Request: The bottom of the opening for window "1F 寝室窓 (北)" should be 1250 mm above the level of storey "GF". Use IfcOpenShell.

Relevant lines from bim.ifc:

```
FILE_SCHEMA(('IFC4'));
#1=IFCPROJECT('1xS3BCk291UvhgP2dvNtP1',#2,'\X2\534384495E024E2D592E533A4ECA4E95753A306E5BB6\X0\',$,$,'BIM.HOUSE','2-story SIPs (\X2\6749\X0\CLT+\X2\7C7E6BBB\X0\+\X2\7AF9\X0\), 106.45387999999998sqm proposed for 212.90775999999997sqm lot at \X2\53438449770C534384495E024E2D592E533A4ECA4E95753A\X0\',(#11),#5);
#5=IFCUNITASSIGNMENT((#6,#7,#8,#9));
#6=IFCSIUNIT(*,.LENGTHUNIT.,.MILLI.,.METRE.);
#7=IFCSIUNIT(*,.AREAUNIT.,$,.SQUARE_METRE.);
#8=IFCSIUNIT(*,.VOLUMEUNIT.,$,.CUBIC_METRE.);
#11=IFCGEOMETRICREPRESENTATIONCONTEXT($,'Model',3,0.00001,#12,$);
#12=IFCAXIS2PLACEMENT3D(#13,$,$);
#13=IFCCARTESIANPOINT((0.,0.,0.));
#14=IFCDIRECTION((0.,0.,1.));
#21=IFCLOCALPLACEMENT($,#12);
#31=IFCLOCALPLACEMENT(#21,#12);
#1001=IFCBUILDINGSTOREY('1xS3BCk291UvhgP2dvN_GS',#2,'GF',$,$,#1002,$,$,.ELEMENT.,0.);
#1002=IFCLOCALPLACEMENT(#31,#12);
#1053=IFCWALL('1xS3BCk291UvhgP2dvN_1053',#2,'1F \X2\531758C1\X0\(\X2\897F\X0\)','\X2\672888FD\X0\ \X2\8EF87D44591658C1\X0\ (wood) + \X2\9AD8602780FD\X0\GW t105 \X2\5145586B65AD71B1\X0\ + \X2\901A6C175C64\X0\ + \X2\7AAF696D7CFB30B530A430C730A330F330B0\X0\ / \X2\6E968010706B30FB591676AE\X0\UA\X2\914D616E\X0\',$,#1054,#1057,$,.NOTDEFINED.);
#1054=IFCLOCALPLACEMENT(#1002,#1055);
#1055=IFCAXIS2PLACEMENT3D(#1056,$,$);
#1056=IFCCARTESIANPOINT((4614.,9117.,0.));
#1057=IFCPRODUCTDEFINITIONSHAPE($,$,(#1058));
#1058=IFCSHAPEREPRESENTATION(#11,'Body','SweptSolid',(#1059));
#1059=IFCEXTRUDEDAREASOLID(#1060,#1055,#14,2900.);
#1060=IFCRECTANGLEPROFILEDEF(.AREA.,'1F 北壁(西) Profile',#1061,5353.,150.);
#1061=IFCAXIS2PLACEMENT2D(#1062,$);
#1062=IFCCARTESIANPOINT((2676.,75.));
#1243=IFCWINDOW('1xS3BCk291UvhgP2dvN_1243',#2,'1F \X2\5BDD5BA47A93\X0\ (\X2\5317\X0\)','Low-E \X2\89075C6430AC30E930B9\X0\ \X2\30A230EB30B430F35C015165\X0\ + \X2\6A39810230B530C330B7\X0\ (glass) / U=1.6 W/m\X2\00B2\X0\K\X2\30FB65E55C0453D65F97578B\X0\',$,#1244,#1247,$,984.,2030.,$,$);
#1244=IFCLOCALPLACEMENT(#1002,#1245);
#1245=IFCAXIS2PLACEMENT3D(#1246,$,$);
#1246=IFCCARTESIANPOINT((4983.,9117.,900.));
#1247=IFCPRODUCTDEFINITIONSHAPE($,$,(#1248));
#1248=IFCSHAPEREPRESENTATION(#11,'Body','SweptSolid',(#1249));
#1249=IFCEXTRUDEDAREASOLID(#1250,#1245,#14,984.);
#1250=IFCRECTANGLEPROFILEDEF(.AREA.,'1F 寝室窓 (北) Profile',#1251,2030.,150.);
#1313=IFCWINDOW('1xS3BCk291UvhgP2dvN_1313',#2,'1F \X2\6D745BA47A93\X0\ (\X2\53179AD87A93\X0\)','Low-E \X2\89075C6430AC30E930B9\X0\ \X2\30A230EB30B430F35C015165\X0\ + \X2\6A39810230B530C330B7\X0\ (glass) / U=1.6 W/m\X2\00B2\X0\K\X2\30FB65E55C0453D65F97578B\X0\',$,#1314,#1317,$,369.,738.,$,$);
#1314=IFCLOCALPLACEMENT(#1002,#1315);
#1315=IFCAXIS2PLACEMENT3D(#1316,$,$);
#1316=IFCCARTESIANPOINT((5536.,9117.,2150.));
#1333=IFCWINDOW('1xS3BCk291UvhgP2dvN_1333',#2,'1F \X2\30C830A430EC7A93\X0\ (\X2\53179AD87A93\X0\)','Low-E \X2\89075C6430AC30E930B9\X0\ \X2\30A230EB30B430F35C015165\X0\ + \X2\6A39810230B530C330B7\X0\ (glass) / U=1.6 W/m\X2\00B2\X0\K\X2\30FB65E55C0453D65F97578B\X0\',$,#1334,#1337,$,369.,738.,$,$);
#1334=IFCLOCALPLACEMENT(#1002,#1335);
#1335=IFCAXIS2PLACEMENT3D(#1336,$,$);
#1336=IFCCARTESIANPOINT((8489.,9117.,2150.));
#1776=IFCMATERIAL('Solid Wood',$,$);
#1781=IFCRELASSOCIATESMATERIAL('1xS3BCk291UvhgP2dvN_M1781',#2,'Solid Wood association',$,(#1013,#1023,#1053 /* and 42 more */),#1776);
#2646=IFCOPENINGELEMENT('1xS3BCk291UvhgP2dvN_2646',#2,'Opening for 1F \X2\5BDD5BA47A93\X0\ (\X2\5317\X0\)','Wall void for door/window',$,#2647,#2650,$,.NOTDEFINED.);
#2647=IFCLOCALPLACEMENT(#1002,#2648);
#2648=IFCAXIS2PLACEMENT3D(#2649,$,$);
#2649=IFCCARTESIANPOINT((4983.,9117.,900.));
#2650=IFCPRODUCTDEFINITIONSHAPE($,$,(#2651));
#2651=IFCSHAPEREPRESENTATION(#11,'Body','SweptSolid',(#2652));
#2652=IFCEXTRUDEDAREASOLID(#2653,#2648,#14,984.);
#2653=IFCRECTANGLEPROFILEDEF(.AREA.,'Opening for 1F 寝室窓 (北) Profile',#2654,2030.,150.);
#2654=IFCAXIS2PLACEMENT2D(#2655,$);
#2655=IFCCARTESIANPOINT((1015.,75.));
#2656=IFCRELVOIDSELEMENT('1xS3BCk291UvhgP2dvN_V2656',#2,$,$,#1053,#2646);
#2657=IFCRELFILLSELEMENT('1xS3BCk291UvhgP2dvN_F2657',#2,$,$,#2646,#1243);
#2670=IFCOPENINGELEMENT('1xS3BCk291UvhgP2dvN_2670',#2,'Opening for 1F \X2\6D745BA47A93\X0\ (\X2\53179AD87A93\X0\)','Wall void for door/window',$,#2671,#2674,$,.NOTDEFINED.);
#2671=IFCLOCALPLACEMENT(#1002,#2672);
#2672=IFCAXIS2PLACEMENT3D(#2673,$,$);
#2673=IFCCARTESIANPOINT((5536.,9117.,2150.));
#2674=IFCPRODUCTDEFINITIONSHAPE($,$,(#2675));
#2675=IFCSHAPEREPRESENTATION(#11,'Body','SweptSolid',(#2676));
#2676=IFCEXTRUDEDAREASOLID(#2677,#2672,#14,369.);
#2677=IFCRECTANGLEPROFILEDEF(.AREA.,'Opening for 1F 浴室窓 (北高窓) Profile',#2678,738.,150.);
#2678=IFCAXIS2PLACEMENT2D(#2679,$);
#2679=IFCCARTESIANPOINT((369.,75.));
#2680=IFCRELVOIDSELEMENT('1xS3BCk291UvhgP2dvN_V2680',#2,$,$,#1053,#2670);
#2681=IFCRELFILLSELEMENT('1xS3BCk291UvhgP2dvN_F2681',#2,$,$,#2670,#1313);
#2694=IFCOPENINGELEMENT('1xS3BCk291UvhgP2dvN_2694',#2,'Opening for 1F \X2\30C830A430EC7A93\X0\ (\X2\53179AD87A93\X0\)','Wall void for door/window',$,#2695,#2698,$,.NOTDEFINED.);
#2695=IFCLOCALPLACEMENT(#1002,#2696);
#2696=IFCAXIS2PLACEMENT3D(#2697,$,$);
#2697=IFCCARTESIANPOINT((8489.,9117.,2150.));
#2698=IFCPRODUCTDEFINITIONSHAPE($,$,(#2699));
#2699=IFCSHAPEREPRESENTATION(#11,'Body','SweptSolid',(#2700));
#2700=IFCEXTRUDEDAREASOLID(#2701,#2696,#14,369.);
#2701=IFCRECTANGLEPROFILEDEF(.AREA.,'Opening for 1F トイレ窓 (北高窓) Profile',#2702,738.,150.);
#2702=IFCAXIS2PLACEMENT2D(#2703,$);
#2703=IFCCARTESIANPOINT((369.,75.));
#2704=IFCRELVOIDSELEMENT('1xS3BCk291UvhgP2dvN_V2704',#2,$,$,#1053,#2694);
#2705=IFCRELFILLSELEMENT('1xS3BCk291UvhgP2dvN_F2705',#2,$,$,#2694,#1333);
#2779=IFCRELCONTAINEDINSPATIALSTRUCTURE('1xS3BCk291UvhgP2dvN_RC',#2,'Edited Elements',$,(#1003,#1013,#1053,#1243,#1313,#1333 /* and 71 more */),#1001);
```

```python
import numpy as np
import ifcopenshell
import ifcopenshell.api.geometry
import ifcopenshell.geom
import ifcopenshell.util.element
import ifcopenshell.util.placement
import ifcopenshell.util.shape
import ifcopenshell.util.unit

model = ifcopenshell.open("bim.ifc")
unit_scale = ifcopenshell.util.unit.calculate_unit_scale(model)

window = model.by_guid("1xS3BCk291UvhgP2dvN_1243")
opening = window.FillsVoids[0].RelatingOpeningElement
storey = ifcopenshell.util.element.get_container(window, ifc_class="IfcBuildingStorey")
level = ifcopenshell.util.placement.get_local_placement(storey.ObjectPlacement)[2, 3]

# The opening's origin need not be at the sill, so measure its lowest point.
shape = ifcopenshell.geom.create_shape(ifcopenshell.geom.settings(), opening)
bottom = ifcopenshell.util.shape.get_shape_bottom_elevation(shape, shape.geometry) / unit_scale
dz = level + 1.25 / unit_scale - bottom

shift = np.array([0.0, 0.0, dz])
# The window is not placed relative to its opening, so move both.
for product in (opening, window):
    matrix = ifcopenshell.util.placement.get_local_placement(product.ObjectPlacement)
    matrix[:3, 3] += shift
    ifcopenshell.api.geometry.edit_object_placement(model, product=product, matrix=matrix, is_si=False)

print(f"moved by {dz * unit_scale:+.3f} m")

model.write("bim_v2.ifc")
```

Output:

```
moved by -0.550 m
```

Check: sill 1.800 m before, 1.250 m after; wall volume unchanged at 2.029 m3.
